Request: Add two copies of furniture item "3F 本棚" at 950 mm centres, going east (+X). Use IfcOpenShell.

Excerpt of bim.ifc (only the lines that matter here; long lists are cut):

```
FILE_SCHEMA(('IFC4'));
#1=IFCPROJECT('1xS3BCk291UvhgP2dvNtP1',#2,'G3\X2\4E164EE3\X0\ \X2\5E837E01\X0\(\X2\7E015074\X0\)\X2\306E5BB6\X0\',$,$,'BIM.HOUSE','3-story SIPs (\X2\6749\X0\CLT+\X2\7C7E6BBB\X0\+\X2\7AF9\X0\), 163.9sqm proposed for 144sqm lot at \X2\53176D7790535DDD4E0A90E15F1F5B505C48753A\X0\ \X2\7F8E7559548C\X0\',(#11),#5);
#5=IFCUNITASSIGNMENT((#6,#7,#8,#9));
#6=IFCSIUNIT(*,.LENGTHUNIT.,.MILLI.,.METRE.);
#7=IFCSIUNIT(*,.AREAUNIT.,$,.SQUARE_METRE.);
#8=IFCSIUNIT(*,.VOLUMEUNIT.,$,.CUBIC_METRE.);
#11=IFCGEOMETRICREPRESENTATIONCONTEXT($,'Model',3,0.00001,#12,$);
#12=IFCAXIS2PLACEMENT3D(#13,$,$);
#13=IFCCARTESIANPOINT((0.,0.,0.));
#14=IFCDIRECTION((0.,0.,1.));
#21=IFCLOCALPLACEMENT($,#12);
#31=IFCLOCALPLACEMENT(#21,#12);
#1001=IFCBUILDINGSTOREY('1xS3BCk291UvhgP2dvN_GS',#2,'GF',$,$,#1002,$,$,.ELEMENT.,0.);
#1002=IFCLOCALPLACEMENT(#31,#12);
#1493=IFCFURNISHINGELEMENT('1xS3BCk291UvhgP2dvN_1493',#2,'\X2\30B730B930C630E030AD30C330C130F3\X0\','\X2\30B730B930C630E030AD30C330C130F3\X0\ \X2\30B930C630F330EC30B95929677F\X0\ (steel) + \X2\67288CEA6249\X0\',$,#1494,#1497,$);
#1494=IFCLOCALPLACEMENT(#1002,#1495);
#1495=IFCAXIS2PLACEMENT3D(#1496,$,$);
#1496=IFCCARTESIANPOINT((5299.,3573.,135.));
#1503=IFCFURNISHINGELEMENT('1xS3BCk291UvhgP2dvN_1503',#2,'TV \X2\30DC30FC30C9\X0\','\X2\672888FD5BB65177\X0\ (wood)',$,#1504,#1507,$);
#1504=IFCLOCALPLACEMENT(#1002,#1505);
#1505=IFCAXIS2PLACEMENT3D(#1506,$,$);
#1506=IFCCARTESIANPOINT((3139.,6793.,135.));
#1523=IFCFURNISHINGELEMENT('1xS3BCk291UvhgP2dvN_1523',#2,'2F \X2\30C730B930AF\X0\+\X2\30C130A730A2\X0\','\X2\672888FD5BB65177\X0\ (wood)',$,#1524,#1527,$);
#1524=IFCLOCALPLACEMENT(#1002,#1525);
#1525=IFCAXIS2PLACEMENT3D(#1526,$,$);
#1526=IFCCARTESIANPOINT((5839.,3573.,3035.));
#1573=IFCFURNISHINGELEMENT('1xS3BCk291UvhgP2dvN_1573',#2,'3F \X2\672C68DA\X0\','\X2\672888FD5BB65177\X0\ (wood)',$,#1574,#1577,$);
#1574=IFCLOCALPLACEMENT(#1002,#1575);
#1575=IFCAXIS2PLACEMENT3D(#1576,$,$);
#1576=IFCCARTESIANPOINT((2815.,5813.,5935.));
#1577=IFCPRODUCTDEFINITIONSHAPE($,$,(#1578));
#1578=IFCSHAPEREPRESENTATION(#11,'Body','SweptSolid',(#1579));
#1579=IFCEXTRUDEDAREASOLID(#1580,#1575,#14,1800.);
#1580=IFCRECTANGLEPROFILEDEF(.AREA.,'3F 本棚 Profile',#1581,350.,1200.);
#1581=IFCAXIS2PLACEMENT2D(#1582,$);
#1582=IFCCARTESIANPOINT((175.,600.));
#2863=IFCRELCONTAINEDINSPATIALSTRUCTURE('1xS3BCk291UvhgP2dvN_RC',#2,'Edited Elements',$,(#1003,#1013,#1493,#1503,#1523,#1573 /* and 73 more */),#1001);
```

```python
import numpy as np
import ifcopenshell
import ifcopenshell.api.geometry
import ifcopenshell.api.root
import ifcopenshell.util.element
import ifcopenshell.util.placement

model = ifcopenshell.open("bim.ifc")


def reuse_history(source, copy):
    """copy_class also copies each property set's owner history, people and application; keep the originals."""
    for rel in copy.IsDefinedBy:
        if rel.is_a("IfcRelDefinesByProperties") and (history := rel.RelatingPropertyDefinition.OwnerHistory):
            rel.RelatingPropertyDefinition.OwnerHistory = source.OwnerHistory
            ifcopenshell.util.element.remove_deep2(model, history)


source = model.by_guid("1xS3BCk291UvhgP2dvN_1573")
base = ifcopenshell.util.placement.get_local_placement(source.ObjectPlacement)
step = np.array([1.0, 0.0, 0.0]) * 950.0

for i in range(1, 3):
    copy = ifcopenshell.api.root.copy_class(model, product=source)
    copy.Representation = ifcopenshell.util.element.copy_deep(
        model, source.Representation, exclude=["IfcGeometricRepresentationContext", "IfcRepresentationMap"]
    )
    reuse_history(source, copy)
    matrix = base.copy()
    matrix[:3, 3] += i * step
    print("added at", matrix[:3, 3].round(3) + 0.0)
    ifcopenshell.api.geometry.edit_object_placement(model, product=copy, matrix=matrix, is_si=False)

model.write("bim_v2.ifc")
```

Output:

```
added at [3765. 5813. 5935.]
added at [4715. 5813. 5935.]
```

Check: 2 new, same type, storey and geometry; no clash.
